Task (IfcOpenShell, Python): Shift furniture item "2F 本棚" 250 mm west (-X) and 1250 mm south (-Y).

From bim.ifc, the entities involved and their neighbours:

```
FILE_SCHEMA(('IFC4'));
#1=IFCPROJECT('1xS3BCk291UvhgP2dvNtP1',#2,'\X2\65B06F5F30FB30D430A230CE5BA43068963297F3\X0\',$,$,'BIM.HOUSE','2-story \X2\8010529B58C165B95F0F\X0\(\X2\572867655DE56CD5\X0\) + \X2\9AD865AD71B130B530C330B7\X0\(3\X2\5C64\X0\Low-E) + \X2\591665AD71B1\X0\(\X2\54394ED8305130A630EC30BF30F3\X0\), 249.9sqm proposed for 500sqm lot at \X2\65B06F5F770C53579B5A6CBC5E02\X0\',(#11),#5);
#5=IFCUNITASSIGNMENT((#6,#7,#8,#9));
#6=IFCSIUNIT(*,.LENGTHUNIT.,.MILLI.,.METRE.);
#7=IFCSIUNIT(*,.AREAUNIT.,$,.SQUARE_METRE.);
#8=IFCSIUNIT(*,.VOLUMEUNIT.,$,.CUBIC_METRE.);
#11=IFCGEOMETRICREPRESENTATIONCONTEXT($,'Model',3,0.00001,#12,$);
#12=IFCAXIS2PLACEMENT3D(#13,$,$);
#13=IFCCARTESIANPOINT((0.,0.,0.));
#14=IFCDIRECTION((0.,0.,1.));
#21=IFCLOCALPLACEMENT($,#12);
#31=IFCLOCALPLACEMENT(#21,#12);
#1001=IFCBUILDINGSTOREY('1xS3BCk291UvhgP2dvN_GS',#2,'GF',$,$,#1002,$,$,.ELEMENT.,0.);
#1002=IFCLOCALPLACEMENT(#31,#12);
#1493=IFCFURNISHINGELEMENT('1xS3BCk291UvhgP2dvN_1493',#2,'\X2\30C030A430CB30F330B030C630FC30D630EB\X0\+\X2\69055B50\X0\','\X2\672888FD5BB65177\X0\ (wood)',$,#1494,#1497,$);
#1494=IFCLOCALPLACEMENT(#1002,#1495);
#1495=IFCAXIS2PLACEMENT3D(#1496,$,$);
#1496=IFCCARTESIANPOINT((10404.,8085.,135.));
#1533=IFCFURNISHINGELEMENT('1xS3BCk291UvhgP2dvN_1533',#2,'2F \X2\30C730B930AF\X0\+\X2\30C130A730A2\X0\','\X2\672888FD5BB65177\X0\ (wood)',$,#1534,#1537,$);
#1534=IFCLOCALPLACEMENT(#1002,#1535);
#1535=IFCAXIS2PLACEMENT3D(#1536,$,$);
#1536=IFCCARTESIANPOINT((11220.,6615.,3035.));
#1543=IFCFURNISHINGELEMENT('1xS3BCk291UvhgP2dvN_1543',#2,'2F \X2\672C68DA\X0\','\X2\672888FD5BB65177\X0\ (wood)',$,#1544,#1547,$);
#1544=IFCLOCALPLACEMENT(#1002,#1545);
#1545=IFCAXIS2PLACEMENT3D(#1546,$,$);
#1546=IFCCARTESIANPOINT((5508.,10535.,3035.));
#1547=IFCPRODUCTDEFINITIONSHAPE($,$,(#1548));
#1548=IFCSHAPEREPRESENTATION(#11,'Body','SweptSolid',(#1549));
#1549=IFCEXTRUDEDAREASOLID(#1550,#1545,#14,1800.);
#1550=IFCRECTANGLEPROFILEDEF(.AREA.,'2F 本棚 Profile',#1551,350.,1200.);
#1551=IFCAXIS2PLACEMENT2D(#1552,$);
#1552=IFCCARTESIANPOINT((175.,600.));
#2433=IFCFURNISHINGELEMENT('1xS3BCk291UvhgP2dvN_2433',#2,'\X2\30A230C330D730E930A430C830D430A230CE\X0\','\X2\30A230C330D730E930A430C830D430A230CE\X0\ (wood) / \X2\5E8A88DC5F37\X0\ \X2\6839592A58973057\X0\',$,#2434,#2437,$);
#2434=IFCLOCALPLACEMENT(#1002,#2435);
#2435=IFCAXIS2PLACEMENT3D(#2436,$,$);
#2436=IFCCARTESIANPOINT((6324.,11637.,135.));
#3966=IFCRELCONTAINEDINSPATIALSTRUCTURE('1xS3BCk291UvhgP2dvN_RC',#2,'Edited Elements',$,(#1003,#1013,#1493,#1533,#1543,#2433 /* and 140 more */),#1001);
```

```python
import ifcopenshell
import ifcopenshell.api.geometry
import ifcopenshell.util.placement
import ifcopenshell.util.unit

model = ifcopenshell.open("bim.ifc")
unit_scale = ifcopenshell.util.unit.calculate_unit_scale(model)

item = model.by_id(1543)
matrix = ifcopenshell.util.placement.get_local_placement(item.ObjectPlacement)
matrix[0, 3] -= 0.25 / unit_scale
matrix[1, 3] -= 1.25 / unit_scale
ifcopenshell.api.geometry.edit_object_placement(model, product=item, matrix=matrix, is_si=False)

print(ifcopenshell.util.placement.get_local_placement(item.ObjectPlacement).round(3) + 0.0)

model.write("bim_v2.ifc")
```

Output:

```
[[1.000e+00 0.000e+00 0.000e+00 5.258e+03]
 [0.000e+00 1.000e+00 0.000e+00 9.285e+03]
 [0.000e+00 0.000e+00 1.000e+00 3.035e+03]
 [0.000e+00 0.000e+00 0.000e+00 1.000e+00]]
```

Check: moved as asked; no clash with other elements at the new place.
